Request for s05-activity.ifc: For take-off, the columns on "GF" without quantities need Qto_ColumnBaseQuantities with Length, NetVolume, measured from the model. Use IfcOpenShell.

First a look at what the model holds.

```python
import ifcopenshell
import ifcopenshell.util.element
import ifcopenshell.util.unit

model = ifcopenshell.open("s05-activity.ifc")
print(model.schema)
for unit_type in ("LENGTHUNIT", "AREAUNIT", "VOLUMEUNIT"):
    print(unit_type, ifcopenshell.util.unit.calculate_unit_scale(model, unit_type))
storey = next(s for s in model.by_type("IfcBuildingStorey") if s.Name == "GF")
columns = [e for e in ifcopenshell.util.element.get_decomposition(storey) if e.is_a("IfcColumn")]
for e in sorted(columns, key=lambda e: e.id()):
    print(e.id(), e.is_a(), e.Name, list(ifcopenshell.util.element.get_psets(e, qtos_only=True)), sep=" | ")
```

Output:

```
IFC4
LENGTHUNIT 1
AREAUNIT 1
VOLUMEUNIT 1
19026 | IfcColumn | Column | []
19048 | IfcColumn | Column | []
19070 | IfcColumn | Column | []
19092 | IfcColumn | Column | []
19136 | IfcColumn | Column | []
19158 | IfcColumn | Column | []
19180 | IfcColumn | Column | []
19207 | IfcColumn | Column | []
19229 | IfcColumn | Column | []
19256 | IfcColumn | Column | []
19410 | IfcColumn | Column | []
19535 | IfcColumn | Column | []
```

```python
import ifcopenshell
import ifcopenshell.api.pset
import ifcopenshell.geom
import ifcopenshell.util.element
import ifcopenshell.util.shape
import ifcopenshell.util.unit

model = ifcopenshell.open("s05-activity.ifc")
unit_scale = ifcopenshell.util.unit.calculate_unit_scale(model)
volume_scale = ifcopenshell.util.unit.calculate_unit_scale(model, "VOLUMEUNIT")
settings = ifcopenshell.geom.settings()

storey = next(s for s in model.by_type("IfcBuildingStorey") if s.Name == "GF")
columns = [e for e in ifcopenshell.util.element.get_decomposition(storey) if e.is_a("IfcColumn")]

for e in sorted(columns, key=lambda e: e.id()):
    if ifcopenshell.util.element.get_psets(e, qtos_only=True, should_inherit=False):
        continue
    # Geometry comes back in metres, in the element's own axes.
    shape = ifcopenshell.geom.create_shape(settings, e)
    values = {
        "Length": ifcopenshell.util.shape.get_z(shape.geometry) / unit_scale,
        "NetVolume": ifcopenshell.util.shape.get_volume(shape.geometry) / volume_scale,
    }
    qto = ifcopenshell.api.pset.add_qto(model, product=e, name="Qto_ColumnBaseQuantities")
    ifcopenshell.api.pset.edit_qto(model, qto=qto, properties=values)
    print(e.id(), {k: round(v, 3) for k, v in values.items()})

model.write("s05-activity_updated.ifc")
```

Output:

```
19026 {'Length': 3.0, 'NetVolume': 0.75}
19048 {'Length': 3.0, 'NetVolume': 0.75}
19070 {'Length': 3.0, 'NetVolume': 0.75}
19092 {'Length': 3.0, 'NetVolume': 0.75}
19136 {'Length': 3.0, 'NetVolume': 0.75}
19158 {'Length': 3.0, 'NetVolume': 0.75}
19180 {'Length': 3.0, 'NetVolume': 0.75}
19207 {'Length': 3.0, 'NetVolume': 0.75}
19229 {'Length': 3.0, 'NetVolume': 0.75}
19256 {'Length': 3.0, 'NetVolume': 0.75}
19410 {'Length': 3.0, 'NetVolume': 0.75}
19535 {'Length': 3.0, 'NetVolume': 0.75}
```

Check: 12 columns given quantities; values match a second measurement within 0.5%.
